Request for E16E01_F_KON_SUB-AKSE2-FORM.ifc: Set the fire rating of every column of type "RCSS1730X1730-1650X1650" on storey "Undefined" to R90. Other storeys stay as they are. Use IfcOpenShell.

First a look at what the model holds.

```python
import ifcopenshell
import ifcopenshell.util.element

model = ifcopenshell.open("E16E01_F_KON_SUB-AKSE2-FORM.ifc")
print(model.schema)
storey = next(s for s in model.by_type("IfcBuildingStorey") if s.Name == "Undefined")
columns = [e for e in ifcopenshell.util.element.get_decomposition(storey) if e.is_a("IfcColumn")]
seen = {}
for e in columns:
    element_type = ifcopenshell.util.element.get_type(e)
    key = (element_type.Name if element_type != e and element_type else None, ifcopenshell.util.element.get_pset(e, "Pset_ColumnCommon", "FireRating"))
    seen[key] = seen.get(key, 0) + 1
for (name, value), count in sorted(seen.items(), key=str):
    print(count, "x", name, "|", value)
```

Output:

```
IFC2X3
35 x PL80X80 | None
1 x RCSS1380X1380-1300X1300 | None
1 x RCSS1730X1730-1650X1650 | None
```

```python
import ifcopenshell
import ifcopenshell.api.pset
import ifcopenshell.util.element

model = ifcopenshell.open("E16E01_F_KON_SUB-AKSE2-FORM.ifc")

storey = next(s for s in model.by_type("IfcBuildingStorey") if s.Name == "Undefined")
columns = [e for e in ifcopenshell.util.element.get_decomposition(storey) if e.is_a("IfcColumn")]

count = 0
for e in columns:
    element_type = ifcopenshell.util.element.get_type(e)
    if element_type in (None, e) or element_type.Name != "RCSS1730X1730-1650X1650":
        continue
    # add_pset returns the element's existing set when there is one.
    pset = ifcopenshell.api.pset.add_pset(model, product=e, name="Pset_ColumnCommon")
    ifcopenshell.api.pset.edit_pset(model, pset=pset, properties={"FireRating": "R90"})
    count += 1

print(count, "columns updated")

model.write("E16E01_F_KON_SUB-AKSE2-FORM-out.ifc")
```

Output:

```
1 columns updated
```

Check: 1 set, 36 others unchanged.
